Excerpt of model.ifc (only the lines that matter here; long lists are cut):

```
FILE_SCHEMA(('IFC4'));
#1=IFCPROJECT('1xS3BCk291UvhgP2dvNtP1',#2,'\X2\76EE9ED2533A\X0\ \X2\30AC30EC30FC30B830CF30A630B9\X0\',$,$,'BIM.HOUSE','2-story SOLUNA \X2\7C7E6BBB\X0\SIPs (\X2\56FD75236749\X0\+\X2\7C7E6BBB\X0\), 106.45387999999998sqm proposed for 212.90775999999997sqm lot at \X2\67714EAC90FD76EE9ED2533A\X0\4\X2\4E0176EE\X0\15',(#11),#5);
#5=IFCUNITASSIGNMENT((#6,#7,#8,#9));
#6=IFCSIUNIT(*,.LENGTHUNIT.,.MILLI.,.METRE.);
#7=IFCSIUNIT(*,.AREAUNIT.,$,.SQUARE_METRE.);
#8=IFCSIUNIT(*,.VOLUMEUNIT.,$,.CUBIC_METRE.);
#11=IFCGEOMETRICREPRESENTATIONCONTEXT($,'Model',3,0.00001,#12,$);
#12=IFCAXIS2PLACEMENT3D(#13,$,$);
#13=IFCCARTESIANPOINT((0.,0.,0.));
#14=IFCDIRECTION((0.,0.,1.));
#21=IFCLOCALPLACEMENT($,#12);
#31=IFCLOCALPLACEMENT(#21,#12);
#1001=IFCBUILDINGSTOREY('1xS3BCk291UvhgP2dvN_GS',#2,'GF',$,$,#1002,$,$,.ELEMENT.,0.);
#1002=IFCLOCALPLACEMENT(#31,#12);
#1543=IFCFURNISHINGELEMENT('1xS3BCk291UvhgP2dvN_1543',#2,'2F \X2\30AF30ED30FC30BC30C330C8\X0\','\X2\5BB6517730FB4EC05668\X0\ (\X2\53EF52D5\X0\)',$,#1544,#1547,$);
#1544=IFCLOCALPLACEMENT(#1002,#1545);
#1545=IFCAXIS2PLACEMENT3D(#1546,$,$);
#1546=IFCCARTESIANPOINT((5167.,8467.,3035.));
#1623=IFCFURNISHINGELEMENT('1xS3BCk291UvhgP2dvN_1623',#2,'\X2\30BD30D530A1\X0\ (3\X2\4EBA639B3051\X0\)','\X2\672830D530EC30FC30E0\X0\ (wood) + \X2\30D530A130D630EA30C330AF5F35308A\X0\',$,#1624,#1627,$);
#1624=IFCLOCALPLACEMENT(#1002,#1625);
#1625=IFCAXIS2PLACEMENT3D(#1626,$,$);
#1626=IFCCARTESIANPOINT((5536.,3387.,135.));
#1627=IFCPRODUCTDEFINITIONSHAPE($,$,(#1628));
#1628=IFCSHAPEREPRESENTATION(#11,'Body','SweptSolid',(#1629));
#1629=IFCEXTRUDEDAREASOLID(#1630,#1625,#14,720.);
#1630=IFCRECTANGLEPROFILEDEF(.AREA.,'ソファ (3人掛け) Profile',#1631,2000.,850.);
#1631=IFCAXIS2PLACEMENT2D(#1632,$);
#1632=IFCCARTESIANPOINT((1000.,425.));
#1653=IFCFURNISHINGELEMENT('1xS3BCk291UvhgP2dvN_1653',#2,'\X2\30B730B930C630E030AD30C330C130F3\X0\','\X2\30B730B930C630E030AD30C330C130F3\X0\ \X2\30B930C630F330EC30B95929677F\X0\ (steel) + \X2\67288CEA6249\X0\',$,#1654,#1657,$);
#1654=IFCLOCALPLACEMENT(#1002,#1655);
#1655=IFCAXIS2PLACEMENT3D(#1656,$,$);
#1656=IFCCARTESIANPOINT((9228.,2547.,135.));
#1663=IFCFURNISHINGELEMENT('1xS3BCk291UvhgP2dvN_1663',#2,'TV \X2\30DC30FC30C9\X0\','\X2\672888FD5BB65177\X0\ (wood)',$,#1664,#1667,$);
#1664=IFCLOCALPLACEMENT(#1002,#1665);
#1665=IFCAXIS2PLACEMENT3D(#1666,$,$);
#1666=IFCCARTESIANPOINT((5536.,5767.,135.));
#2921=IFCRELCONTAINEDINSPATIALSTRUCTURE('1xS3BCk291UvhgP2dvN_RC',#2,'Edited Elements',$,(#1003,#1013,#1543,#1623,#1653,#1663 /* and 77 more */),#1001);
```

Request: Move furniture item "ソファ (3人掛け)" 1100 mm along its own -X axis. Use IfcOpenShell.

```python
import ifcopenshell
import ifcopenshell.api.geometry
import ifcopenshell.util.placement
import ifcopenshell.util.unit

model = ifcopenshell.open("model.ifc")
unit_scale = ifcopenshell.util.unit.calculate_unit_scale(model)

item = model.by_guid("1xS3BCk291UvhgP2dvN_1623")
matrix = ifcopenshell.util.placement.get_local_placement(item.ObjectPlacement)
matrix[:3, 3] -= matrix[:3, 0] * 1.1 / unit_scale
ifcopenshell.api.geometry.edit_object_placement(model, product=item, matrix=matrix, is_si=False)

print(ifcopenshell.util.placement.get_local_placement(item.ObjectPlacement).round(3) + 0.0)

model.write("model_rev.ifc")
```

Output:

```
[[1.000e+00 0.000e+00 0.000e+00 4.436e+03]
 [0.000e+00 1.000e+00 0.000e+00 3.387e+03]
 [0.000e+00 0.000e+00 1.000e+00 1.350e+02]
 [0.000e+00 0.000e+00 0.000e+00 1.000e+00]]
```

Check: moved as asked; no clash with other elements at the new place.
